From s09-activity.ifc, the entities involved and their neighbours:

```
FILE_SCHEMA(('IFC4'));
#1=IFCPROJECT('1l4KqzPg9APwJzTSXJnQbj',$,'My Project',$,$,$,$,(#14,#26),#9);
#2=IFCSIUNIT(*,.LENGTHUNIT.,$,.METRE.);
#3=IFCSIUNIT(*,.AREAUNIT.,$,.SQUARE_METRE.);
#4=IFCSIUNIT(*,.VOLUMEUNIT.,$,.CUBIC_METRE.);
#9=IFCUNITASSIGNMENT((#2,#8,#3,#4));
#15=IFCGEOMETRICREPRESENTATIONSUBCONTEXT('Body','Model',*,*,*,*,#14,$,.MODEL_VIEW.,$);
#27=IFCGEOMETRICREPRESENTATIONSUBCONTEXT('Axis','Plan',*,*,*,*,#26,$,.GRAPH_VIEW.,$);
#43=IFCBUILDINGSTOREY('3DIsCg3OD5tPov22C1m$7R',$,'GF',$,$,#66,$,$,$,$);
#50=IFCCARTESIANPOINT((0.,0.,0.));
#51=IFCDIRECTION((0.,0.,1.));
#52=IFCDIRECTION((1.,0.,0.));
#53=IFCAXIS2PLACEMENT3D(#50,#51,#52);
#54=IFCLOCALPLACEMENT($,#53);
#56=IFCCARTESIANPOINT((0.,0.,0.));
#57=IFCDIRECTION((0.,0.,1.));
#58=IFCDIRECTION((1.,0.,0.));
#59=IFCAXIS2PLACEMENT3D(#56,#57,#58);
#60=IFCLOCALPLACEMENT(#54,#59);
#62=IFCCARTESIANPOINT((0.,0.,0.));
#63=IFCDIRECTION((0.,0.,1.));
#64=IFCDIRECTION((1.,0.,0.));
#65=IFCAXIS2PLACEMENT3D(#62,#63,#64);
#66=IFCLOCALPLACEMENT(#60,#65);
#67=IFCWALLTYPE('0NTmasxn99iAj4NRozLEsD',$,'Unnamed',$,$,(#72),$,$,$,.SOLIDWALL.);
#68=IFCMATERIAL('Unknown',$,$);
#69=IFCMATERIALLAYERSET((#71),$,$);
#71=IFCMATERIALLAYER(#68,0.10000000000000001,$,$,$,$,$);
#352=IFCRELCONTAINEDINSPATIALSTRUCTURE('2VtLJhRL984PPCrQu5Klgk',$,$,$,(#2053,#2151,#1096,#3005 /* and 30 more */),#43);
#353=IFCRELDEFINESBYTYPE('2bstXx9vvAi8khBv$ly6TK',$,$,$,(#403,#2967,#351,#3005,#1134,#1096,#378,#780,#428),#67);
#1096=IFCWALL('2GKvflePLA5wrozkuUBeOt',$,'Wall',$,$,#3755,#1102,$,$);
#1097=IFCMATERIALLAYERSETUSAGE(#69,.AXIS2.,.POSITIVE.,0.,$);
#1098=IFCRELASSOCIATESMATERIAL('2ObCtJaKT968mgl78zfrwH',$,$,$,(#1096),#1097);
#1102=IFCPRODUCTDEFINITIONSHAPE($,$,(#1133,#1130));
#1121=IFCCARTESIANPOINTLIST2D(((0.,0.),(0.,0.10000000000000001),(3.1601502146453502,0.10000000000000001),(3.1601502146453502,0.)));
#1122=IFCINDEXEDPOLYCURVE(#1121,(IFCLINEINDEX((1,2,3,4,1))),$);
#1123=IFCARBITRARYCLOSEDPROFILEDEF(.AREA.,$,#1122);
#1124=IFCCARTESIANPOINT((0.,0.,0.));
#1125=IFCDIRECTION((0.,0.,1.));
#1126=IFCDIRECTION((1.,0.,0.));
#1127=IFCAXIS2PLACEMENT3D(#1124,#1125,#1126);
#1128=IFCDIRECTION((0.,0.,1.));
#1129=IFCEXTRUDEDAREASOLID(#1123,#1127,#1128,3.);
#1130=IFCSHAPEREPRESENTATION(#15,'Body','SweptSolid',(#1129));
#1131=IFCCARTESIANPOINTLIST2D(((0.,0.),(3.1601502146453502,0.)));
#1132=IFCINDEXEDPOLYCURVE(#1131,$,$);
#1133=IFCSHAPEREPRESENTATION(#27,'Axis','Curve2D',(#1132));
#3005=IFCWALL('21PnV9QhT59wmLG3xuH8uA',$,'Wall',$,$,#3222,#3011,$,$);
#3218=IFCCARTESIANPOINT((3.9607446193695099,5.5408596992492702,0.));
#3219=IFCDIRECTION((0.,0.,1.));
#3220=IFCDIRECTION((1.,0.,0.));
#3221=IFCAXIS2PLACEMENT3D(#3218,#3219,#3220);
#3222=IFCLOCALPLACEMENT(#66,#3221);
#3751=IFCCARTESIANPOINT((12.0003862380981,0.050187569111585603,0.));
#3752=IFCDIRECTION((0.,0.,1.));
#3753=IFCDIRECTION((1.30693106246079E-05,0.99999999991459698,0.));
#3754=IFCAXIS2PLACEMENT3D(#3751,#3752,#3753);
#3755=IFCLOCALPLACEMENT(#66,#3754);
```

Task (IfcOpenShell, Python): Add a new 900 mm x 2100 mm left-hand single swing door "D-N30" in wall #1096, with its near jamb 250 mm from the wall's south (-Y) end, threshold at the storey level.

```python
import numpy as np
import ifcopenshell
import ifcopenshell.api.feature
import ifcopenshell.api.geometry
import ifcopenshell.api.root
import ifcopenshell.api.spatial
import ifcopenshell.geom
import ifcopenshell.util.element
import ifcopenshell.util.placement
import ifcopenshell.util.representation
import ifcopenshell.util.shape
import ifcopenshell.util.unit

model = ifcopenshell.open("s09-activity.ifc")
unit_scale = ifcopenshell.util.unit.calculate_unit_scale(model)
settings = ifcopenshell.geom.settings()


def volume(element):
    """Net volume in cubic metres, openings subtracted."""
    shape = ifcopenshell.geom.create_shape(settings, element)
    return ifcopenshell.util.shape.get_volume(shape.geometry)


wall = model.by_guid("2GKvflePLA5wrozkuUBeOt")
storey = ifcopenshell.util.element.get_container(wall, ifc_class="IfcBuildingStorey")
context = ifcopenshell.util.representation.get_context(model, "Model", "Body", "MODEL_VIEW")
before = volume(wall)

width, height, from_end, sill = 0.9, 2.1, 0.25, 0.0  # metres

# The wall runs along its own X axis, and the end named is its -X end.
wall_shape = ifcopenshell.geom.create_shape(settings, wall)
x, y, z = ifcopenshell.util.shape.get_vertices(wall_shape.geometry).T
start = x.min() + from_end
face, thickness = float(y.min()), float(y.max() - y.min())
wall_matrix = ifcopenshell.util.placement.get_local_placement(wall.ObjectPlacement)
level = ifcopenshell.util.placement.get_local_placement(storey.ObjectPlacement)[2, 3]


def in_wall(x, y):
    """Placement at x, y metres in the wall's axes, at sill height."""
    matrix = wall_matrix.copy()
    matrix[:, 3] = wall_matrix @ np.array([x / unit_scale, y / unit_scale, 0.0, 1.0])
    matrix[2, 3] = level + sill / unit_scale
    return matrix


# Opening: a box that overshoots both wall faces by 50 mm.
opening = ifcopenshell.api.root.create_entity(model, ifc_class="IfcOpeningElement", predefined_type="OPENING")
box = ifcopenshell.api.geometry.add_wall_representation(
    model, context=context, length=width, height=height, thickness=thickness + 0.1
)
ifcopenshell.api.geometry.assign_representation(model, product=opening, representation=box)
ifcopenshell.api.geometry.edit_object_placement(model, product=opening, matrix=in_wall(start, face - 0.05), is_si=False)
ifcopenshell.api.feature.add_feature(model, feature=opening, element=wall)

door = ifcopenshell.api.root.create_entity(model, ifc_class="IfcDoor", name="D-N30", predefined_type="DOOR")
door.OverallWidth, door.OverallHeight = width / unit_scale, height / unit_scale
door.OperationType = "SINGLE_SWING_LEFT"
body = ifcopenshell.api.geometry.add_door_representation(
    model,
    context=context,
    overall_width=door.OverallWidth,
    overall_height=door.OverallHeight,
    operation_type="SINGLE_SWING_LEFT",
    lining_properties={"LiningDepth": thickness / unit_scale, "ThresholdDepth": thickness / unit_scale},
)
ifcopenshell.api.geometry.assign_representation(model, product=door, representation=body)
ifcopenshell.api.spatial.assign_container(model, products=[door], relating_structure=storey)
ifcopenshell.api.feature.add_filling(model, opening=opening, element=door)

# The lining spans the wall, so the door starts at the wall face.
ifcopenshell.api.geometry.edit_object_placement(model, product=door, matrix=in_wall(start, face), is_si=False)

after = volume(wall)

print(f"wall volume {before:.3f} -> {after:.3f} m3")

model.write("s09-activity_edited.ifc")
```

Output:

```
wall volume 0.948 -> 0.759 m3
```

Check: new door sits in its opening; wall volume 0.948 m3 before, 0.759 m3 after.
